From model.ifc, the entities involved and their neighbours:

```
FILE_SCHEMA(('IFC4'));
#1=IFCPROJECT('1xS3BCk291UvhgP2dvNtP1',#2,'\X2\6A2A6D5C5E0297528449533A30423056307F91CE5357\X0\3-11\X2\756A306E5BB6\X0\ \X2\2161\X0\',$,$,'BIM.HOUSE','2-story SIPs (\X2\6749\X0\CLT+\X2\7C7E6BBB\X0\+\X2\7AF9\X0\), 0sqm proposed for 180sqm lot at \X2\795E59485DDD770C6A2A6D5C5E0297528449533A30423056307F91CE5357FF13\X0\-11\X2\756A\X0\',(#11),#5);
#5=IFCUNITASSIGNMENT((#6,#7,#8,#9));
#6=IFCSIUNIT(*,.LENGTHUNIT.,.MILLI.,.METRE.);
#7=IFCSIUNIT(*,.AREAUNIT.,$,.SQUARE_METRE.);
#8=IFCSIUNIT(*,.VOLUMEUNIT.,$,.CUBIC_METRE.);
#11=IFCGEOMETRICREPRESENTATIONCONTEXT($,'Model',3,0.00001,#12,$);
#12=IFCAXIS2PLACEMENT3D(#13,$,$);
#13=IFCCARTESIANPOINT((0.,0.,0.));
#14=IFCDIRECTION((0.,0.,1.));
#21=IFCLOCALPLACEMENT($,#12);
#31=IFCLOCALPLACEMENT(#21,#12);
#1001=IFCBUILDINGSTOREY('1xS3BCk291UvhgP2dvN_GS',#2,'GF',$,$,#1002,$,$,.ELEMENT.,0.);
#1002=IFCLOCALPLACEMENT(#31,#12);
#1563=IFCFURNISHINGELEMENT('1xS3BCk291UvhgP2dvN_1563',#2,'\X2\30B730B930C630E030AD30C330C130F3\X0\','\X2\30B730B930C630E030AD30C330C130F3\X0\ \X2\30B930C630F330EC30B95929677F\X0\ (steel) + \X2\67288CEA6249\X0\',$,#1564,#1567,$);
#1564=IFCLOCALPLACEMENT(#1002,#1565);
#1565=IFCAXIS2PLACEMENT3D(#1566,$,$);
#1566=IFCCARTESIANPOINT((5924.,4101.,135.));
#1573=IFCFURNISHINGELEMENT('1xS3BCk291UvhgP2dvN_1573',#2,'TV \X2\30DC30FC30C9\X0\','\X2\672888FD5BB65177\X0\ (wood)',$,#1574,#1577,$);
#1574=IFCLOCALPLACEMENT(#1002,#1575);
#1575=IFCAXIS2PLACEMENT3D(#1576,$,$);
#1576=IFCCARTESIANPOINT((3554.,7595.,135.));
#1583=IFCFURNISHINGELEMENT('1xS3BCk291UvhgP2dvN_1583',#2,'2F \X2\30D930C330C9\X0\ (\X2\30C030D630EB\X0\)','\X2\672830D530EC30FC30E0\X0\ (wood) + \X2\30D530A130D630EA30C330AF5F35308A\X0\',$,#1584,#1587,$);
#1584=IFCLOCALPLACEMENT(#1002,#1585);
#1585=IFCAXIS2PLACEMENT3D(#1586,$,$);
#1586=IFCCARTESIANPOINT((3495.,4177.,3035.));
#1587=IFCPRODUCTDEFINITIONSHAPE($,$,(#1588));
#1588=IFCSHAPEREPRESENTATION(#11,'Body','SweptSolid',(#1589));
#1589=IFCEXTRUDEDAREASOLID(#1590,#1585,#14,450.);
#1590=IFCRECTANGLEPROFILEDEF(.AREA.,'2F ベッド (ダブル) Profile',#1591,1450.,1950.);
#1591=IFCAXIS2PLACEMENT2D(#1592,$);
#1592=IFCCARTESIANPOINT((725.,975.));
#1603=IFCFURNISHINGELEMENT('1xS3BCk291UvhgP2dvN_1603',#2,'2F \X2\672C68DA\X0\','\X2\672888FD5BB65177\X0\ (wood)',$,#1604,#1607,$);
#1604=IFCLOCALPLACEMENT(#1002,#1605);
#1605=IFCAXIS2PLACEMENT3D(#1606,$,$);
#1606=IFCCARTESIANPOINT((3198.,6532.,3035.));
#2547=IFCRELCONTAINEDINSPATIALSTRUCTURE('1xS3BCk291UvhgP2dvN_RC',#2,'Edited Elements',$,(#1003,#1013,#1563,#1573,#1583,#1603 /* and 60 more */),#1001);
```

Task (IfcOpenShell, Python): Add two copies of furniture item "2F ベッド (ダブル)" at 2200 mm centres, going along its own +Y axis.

```python
import ifcopenshell
import ifcopenshell.api.geometry
import ifcopenshell.api.root
import ifcopenshell.util.element
import ifcopenshell.util.placement
import ifcopenshell.util.unit

model = ifcopenshell.open("model.ifc")
unit_scale = ifcopenshell.util.unit.calculate_unit_scale(model)


def reuse_history(source, copy):
    """copy_class also copies each property set's owner history, people and application; keep the originals."""
    for rel in copy.IsDefinedBy:
        if rel.is_a("IfcRelDefinesByProperties") and (history := rel.RelatingPropertyDefinition.OwnerHistory):
            rel.RelatingPropertyDefinition.OwnerHistory = source.OwnerHistory
            ifcopenshell.util.element.remove_deep2(model, history)


source = model.by_guid("1xS3BCk291UvhgP2dvN_1583")
base = ifcopenshell.util.placement.get_local_placement(source.ObjectPlacement)
step = base[:3, 1] * 2.2 / unit_scale

for i in range(1, 3):
    copy = ifcopenshell.api.root.copy_class(model, product=source)
    copy.Representation = ifcopenshell.util.element.copy_deep(
        model, source.Representation, exclude=["IfcGeometricRepresentationContext", "IfcRepresentationMap"]
    )
    reuse_history(source, copy)
    matrix = base.copy()
    matrix[:3, 3] += i * step
    print("added at", matrix[:3, 3].round(3) + 0.0)
    ifcopenshell.api.geometry.edit_object_placement(model, product=copy, matrix=matrix, is_si=False)

model.write("model_updated.ifc")
```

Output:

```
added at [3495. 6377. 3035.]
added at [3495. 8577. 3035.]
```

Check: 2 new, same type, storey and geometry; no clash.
